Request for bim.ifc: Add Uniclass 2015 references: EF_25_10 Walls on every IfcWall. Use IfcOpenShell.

First a look at what the model holds.

```python
import ifcopenshell

model = ifcopenshell.open("bim.ifc")
print(model.schema)
print("classifications:", [c.Name for c in model.by_type("IfcClassification")])
for ifc_class in ("IfcDoor", "IfcRoof", "IfcStair", "IfcWall", "IfcWindow"):
    print(ifc_class, len(model.by_type(ifc_class)))
```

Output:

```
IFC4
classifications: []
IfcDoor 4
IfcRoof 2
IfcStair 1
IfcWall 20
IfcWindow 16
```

```python
import ifcopenshell
import ifcopenshell.api.classification

model = ifcopenshell.open("bim.ifc")

system = ifcopenshell.api.classification.add_classification(model, classification="Uniclass 2015")

codes = {
    "IfcWall": ("EF_25_10", "Walls"),
}
for ifc_class, (code, name) in codes.items():
    products = model.by_type(ifc_class)
    ifcopenshell.api.classification.add_reference(
        model, products=products, classification=system, identification=code, name=name
    )
    print(code, len(products))

model.write("bim_edited.ifc")
```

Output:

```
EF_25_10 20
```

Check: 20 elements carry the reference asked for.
